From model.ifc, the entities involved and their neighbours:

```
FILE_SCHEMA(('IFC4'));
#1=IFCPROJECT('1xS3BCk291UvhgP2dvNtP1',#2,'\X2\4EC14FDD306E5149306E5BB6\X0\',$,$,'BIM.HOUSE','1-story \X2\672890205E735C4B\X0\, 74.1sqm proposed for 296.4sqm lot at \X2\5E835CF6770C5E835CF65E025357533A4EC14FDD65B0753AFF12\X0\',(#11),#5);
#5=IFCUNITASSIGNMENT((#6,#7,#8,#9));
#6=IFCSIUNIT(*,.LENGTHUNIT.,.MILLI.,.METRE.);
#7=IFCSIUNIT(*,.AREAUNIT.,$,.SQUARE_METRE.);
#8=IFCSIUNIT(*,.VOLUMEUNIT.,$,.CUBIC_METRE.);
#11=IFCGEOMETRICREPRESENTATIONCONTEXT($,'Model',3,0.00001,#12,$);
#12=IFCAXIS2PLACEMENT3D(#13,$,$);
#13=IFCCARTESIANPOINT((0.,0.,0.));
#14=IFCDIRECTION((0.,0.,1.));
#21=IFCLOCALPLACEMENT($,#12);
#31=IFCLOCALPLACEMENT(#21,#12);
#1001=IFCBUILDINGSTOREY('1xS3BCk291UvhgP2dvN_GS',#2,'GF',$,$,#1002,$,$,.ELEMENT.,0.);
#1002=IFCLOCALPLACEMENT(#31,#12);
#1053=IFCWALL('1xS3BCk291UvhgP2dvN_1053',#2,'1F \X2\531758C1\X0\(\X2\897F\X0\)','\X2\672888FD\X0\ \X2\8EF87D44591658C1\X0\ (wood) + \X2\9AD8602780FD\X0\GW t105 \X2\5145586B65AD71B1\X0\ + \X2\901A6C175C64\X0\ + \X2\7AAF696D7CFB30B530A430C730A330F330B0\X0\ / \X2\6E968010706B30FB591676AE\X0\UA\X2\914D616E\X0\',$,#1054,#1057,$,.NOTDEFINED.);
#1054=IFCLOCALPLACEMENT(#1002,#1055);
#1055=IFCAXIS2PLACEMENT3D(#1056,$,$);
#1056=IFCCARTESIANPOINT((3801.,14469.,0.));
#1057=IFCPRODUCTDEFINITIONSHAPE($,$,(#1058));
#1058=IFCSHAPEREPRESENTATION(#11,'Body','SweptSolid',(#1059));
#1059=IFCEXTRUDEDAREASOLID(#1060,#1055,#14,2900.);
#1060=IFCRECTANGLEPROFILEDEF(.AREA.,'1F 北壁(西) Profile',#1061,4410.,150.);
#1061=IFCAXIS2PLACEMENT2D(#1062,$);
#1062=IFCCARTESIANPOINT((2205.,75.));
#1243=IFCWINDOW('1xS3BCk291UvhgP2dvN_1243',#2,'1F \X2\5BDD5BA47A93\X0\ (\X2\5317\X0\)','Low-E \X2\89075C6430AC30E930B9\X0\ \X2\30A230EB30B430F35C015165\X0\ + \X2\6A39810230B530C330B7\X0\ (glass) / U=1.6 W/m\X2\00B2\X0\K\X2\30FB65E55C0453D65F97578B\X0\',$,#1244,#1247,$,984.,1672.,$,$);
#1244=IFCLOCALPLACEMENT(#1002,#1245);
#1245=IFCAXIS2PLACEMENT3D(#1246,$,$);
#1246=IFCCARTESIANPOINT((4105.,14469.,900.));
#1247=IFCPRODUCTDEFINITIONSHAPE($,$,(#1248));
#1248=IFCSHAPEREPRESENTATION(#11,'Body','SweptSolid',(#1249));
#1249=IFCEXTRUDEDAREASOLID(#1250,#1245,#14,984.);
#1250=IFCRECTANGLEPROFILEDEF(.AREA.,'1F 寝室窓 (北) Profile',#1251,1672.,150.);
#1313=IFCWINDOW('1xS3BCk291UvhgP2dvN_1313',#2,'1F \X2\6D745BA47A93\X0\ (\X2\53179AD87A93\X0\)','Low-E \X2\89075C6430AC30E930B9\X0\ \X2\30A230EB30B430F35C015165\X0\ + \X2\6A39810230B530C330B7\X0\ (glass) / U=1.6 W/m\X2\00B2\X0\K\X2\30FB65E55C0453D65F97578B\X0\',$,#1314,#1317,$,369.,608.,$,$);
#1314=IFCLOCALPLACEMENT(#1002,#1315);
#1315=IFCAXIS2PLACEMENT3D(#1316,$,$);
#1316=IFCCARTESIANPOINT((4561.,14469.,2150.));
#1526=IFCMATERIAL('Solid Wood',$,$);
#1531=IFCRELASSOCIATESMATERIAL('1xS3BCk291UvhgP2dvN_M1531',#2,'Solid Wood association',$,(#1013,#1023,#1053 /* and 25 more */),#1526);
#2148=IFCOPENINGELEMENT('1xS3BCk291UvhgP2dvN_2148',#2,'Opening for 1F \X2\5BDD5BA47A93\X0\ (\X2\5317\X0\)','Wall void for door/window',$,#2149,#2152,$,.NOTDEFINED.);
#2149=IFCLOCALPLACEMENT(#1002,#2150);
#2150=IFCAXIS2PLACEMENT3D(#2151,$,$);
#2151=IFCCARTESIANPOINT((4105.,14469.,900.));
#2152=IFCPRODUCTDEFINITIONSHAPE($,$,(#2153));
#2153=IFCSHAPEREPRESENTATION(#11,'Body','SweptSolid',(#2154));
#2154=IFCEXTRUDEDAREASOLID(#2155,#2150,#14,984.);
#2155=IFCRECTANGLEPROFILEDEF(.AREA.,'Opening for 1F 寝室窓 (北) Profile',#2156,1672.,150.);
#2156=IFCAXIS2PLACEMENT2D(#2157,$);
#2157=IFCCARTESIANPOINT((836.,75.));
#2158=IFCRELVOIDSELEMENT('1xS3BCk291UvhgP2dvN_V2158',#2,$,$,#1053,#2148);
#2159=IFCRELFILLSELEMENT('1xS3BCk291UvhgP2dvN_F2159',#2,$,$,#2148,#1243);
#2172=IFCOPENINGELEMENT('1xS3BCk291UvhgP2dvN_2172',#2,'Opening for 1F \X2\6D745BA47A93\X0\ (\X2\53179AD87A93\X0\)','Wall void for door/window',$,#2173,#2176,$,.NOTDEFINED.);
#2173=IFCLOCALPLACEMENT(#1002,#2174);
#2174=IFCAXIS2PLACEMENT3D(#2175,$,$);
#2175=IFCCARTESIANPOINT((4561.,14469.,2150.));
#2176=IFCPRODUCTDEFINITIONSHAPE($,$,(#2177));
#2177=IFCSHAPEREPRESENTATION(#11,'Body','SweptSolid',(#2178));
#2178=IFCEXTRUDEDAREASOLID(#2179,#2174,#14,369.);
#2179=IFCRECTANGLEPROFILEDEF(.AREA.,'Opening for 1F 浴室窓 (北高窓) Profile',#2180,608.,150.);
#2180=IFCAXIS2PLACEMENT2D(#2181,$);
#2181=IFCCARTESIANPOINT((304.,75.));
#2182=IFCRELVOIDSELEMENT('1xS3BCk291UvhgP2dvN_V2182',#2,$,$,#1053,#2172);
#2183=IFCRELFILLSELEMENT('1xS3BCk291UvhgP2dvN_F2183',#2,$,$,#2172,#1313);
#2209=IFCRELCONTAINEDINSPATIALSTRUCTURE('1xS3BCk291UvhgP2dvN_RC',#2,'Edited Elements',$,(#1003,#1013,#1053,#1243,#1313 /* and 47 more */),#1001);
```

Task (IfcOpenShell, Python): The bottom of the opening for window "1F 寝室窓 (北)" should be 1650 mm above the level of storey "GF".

```python
import numpy as np
import ifcopenshell
import ifcopenshell.api.geometry
import ifcopenshell.geom
import ifcopenshell.util.element
import ifcopenshell.util.placement
import ifcopenshell.util.shape
import ifcopenshell.util.unit

model = ifcopenshell.open("model.ifc")
unit_scale = ifcopenshell.util.unit.calculate_unit_scale(model)

window = model.by_id(1243)
opening = window.FillsVoids[0].RelatingOpeningElement
storey = ifcopenshell.util.element.get_container(window, ifc_class="IfcBuildingStorey")
level = ifcopenshell.util.placement.get_local_placement(storey.ObjectPlacement)[2, 3]

# The opening's origin need not be at the sill, so measure its lowest point.
shape = ifcopenshell.geom.create_shape(ifcopenshell.geom.settings(), opening)
bottom = ifcopenshell.util.shape.get_shape_bottom_elevation(shape, shape.geometry) / unit_scale
dz = level + 1.65 / unit_scale - bottom

shift = np.array([0.0, 0.0, dz])
# The window is not placed relative to its opening, so move both.
for product in (opening, window):
    matrix = ifcopenshell.util.placement.get_local_placement(product.ObjectPlacement)
    matrix[:3, 3] += shift
    ifcopenshell.api.geometry.edit_object_placement(model, product=product, matrix=matrix, is_si=False)

print(f"moved by {dz * unit_scale:+.3f} m")

model.write("model_rev.ifc")
```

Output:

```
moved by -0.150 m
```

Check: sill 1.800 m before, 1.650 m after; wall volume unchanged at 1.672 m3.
